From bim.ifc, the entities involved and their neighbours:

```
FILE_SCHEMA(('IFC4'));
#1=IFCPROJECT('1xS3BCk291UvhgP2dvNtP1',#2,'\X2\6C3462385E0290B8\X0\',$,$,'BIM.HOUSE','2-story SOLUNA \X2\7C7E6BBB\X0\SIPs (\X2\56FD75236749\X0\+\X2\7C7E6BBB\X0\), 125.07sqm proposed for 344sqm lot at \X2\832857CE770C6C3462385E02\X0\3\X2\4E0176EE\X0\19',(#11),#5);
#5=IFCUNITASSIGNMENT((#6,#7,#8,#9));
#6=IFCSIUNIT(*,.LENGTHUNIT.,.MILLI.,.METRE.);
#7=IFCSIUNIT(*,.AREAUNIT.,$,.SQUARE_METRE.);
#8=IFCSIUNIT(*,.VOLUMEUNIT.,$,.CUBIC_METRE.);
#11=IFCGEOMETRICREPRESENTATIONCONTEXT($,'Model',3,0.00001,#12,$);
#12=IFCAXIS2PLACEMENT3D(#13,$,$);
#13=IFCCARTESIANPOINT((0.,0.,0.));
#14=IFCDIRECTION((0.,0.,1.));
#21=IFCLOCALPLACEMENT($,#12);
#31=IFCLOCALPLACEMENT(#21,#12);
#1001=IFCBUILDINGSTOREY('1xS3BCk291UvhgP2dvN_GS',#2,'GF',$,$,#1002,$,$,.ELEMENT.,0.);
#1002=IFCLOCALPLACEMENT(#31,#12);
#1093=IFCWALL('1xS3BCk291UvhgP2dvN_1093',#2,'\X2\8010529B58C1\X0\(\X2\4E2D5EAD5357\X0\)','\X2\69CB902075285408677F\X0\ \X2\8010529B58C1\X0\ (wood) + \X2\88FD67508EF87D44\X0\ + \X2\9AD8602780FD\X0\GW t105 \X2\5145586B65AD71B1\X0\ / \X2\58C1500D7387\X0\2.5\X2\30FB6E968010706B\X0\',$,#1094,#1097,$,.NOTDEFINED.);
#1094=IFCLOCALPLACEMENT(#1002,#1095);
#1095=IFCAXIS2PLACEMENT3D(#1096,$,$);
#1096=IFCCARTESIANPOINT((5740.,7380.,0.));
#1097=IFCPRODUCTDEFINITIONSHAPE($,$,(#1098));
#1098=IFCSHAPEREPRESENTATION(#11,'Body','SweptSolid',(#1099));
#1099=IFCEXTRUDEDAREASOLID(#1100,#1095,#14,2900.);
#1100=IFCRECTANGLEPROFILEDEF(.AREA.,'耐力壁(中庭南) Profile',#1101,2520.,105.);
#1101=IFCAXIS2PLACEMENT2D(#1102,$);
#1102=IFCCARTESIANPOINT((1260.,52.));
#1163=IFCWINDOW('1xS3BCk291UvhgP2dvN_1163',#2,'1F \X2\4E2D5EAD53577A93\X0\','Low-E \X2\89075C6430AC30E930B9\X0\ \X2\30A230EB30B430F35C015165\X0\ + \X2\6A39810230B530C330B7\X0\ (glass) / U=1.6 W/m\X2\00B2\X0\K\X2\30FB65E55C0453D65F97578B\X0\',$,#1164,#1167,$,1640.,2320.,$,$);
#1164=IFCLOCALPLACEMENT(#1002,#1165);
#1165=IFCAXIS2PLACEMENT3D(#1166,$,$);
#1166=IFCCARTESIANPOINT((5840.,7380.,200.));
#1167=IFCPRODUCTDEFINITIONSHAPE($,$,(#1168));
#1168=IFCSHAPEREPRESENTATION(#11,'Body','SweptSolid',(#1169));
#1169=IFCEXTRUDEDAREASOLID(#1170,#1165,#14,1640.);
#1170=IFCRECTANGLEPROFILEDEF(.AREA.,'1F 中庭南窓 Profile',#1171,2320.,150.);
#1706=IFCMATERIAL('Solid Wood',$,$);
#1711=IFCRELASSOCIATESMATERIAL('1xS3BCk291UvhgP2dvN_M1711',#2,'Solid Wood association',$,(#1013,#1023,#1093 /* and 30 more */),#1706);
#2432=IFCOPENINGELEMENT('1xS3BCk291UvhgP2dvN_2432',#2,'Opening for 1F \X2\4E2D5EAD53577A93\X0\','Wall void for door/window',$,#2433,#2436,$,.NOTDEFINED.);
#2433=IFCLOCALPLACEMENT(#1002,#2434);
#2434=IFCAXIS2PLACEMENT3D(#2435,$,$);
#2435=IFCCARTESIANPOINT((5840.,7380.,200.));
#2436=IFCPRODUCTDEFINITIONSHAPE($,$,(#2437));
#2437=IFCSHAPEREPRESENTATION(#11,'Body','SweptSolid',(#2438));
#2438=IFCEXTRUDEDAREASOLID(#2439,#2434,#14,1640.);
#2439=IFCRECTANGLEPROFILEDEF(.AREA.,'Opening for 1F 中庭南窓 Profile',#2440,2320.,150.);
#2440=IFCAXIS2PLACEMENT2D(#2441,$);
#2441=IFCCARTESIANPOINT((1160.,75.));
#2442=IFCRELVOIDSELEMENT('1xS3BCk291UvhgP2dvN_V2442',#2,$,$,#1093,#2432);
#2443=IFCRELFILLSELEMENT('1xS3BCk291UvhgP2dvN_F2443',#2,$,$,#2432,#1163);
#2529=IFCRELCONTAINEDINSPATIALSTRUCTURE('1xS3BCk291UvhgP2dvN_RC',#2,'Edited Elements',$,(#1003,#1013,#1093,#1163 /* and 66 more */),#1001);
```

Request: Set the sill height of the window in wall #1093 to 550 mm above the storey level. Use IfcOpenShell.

```python
import numpy as np
import ifcopenshell
import ifcopenshell.api.geometry
import ifcopenshell.geom
import ifcopenshell.util.element
import ifcopenshell.util.placement
import ifcopenshell.util.shape
import ifcopenshell.util.unit

model = ifcopenshell.open("bim.ifc")
unit_scale = ifcopenshell.util.unit.calculate_unit_scale(model)

window = model.by_id(1163)
opening = window.FillsVoids[0].RelatingOpeningElement
storey = ifcopenshell.util.element.get_container(window, ifc_class="IfcBuildingStorey")
level = ifcopenshell.util.placement.get_local_placement(storey.ObjectPlacement)[2, 3]

# The opening's origin need not be at the sill, so measure its lowest point.
shape = ifcopenshell.geom.create_shape(ifcopenshell.geom.settings(), opening)
bottom = ifcopenshell.util.shape.get_shape_bottom_elevation(shape, shape.geometry) / unit_scale
dz = level + 0.55 / unit_scale - bottom

shift = np.array([0.0, 0.0, dz])
# The window is not placed relative to its opening, so move both.
for product in (opening, window):
    matrix = ifcopenshell.util.placement.get_local_placement(product.ObjectPlacement)
    matrix[:3, 3] += shift
    ifcopenshell.api.geometry.edit_object_placement(model, product=product, matrix=matrix, is_si=False)

print(f"moved by {dz * unit_scale:+.3f} m")

model.write("bim-out.ifc")
```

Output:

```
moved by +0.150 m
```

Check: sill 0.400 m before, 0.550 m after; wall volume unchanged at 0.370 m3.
